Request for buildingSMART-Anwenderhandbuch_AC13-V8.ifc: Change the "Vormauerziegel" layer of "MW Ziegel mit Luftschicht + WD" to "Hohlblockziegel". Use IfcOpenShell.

First a look at what the model holds.

```python
import ifcopenshell
import ifcopenshell.util.element

model = ifcopenshell.open("buildingSMART-Anwenderhandbuch_AC13-V8.ifc")
print(model.schema)
for layer_set in model.by_type("IfcMaterialLayerSet"):
    if layer_set.LayerSetName == "MW Ziegel mit Luftschicht + WD":
        for layer in layer_set.MaterialLayers:
            print(layer.id(), layer.Material and layer.Material.Name, layer.LayerThickness, sep=" | ")
        print(len(ifcopenshell.util.element.get_elements_by_material(model, layer_set)), "elements and types use it")
print(sorted(m.Name for m in model.by_type("IfcMaterial") if m.Name)[:60])
```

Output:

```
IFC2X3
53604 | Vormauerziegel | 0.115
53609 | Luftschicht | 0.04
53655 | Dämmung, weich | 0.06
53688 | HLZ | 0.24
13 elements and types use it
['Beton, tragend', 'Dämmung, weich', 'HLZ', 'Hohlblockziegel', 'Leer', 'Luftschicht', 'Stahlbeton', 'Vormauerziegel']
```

```python
import ifcopenshell
import ifcopenshell.api.material

model = ifcopenshell.open("buildingSMART-Anwenderhandbuch_AC13-V8.ifc")

layer_set = next(s for s in model.by_type("IfcMaterialLayerSet") if s.LayerSetName == "MW Ziegel mit Luftschicht + WD")
layer = next(l for l in layer_set.MaterialLayers if l.Material and l.Material.Name == "Vormauerziegel")
material = next(m for m in model.by_type("IfcMaterial") if m.Name == "Hohlblockziegel")

# Point this one layer at the other material; renaming the old one would change it everywhere.
ifcopenshell.api.material.edit_layer(model, layer=layer, attributes={}, material=material)

print([l.Material.Name if l.Material else None for l in layer_set.MaterialLayers])

model.write("buildingSMART-Anwenderhandbuch_AC13-V8_v2.ifc")
```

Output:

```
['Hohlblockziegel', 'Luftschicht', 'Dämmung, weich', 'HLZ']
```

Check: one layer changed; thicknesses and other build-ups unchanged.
